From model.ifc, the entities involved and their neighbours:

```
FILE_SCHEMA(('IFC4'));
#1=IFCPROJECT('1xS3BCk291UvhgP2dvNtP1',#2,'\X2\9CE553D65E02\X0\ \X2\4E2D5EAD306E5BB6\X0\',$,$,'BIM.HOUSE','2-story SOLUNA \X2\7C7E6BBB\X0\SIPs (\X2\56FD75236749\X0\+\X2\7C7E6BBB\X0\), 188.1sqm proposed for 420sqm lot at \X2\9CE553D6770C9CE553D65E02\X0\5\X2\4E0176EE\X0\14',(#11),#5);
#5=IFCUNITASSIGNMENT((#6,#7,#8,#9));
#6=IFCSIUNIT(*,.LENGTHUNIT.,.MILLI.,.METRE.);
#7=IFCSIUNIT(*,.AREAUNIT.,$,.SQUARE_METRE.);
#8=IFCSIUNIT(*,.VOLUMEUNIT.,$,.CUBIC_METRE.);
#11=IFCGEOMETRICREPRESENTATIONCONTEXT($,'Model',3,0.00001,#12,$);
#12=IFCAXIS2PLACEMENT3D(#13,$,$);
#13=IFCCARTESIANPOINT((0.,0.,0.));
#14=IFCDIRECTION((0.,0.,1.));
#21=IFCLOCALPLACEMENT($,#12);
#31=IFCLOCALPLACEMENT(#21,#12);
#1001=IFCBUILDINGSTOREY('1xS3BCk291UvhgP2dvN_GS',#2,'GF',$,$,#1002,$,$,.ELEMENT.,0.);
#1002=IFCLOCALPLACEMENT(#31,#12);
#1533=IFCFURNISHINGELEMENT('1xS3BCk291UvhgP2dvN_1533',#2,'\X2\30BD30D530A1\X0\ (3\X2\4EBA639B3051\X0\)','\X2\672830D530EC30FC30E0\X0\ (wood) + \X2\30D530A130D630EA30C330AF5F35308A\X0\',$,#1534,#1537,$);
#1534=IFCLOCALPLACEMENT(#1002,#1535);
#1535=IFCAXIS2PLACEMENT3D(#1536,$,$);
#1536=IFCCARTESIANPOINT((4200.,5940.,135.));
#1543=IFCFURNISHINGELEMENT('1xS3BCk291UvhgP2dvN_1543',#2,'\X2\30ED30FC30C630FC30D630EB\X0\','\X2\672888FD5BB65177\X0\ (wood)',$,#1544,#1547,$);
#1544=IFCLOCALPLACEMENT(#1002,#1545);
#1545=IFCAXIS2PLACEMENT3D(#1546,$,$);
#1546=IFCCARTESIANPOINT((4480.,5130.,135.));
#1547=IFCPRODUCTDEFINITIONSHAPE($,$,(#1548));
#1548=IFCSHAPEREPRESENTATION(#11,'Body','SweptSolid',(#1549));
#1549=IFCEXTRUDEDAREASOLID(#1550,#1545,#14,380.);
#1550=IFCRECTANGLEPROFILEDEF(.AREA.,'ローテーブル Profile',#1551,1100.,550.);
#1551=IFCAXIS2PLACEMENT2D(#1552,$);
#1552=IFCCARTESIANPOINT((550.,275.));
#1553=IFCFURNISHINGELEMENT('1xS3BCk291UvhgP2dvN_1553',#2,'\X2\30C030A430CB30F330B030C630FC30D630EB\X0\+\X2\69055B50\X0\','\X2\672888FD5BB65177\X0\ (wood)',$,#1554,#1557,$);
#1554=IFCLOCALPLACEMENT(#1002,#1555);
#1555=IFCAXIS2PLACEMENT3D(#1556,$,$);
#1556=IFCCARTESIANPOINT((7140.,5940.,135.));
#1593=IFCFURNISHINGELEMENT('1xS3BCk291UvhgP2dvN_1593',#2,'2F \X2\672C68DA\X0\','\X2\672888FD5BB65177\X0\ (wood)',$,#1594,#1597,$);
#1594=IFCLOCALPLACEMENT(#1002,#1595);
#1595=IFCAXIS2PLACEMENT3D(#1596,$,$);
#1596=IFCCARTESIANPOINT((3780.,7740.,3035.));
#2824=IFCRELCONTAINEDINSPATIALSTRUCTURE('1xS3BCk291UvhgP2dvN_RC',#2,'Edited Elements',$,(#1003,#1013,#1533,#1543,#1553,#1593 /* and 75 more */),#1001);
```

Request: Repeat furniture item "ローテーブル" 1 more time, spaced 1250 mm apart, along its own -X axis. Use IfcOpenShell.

```python
import ifcopenshell
import ifcopenshell.api.geometry
import ifcopenshell.api.root
import ifcopenshell.util.element
import ifcopenshell.util.placement
import ifcopenshell.util.unit

model = ifcopenshell.open("model.ifc")
unit_scale = ifcopenshell.util.unit.calculate_unit_scale(model)


def reuse_history(source, copy):
    """copy_class also copies each property set's owner history, people and application; keep the originals."""
    for rel in copy.IsDefinedBy:
        if rel.is_a("IfcRelDefinesByProperties") and (history := rel.RelatingPropertyDefinition.OwnerHistory):
            rel.RelatingPropertyDefinition.OwnerHistory = source.OwnerHistory
            ifcopenshell.util.element.remove_deep2(model, history)


source = model.by_id(1543)
base = ifcopenshell.util.placement.get_local_placement(source.ObjectPlacement)
step = -base[:3, 0] * 1.25 / unit_scale

for i in range(1, 2):
    copy = ifcopenshell.api.root.copy_class(model, product=source)
    copy.Representation = ifcopenshell.util.element.copy_deep(
        model, source.Representation, exclude=["IfcGeometricRepresentationContext", "IfcRepresentationMap"]
    )
    reuse_history(source, copy)
    matrix = base.copy()
    matrix[:3, 3] += i * step
    print("added at", matrix[:3, 3].round(3) + 0.0)
    ifcopenshell.api.geometry.edit_object_placement(model, product=copy, matrix=matrix, is_si=False)

model.write("model_rev.ifc")
```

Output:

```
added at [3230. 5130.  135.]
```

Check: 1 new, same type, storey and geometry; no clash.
